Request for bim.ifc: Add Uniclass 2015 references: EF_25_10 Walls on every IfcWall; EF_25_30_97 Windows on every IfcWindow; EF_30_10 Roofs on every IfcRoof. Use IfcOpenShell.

First a look at what the model holds.

```python
import ifcopenshell

model = ifcopenshell.open("bim.ifc")
print(model.schema)
print("classifications:", [c.Name for c in model.by_type("IfcClassification")])
for ifc_class in ("IfcDoor", "IfcRoof", "IfcStair", "IfcWall", "IfcWindow"):
    print(ifc_class, len(model.by_type(ifc_class)))
```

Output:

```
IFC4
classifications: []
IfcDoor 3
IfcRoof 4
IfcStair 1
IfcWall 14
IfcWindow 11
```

```python
import ifcopenshell
import ifcopenshell.api.classification

model = ifcopenshell.open("bim.ifc")

system = ifcopenshell.api.classification.add_classification(model, classification="Uniclass 2015")

codes = {
    "IfcWall": ("EF_25_10", "Walls"),
    "IfcWindow": ("EF_25_30_97", "Windows"),
    "IfcRoof": ("EF_30_10", "Roofs"),
}
for ifc_class, (code, name) in codes.items():
    products = model.by_type(ifc_class)
    ifcopenshell.api.classification.add_reference(
        model, products=products, classification=system, identification=code, name=name
    )
    print(code, len(products))

model.write("bim_rev.ifc")
```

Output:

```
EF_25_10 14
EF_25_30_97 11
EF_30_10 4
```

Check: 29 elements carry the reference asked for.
